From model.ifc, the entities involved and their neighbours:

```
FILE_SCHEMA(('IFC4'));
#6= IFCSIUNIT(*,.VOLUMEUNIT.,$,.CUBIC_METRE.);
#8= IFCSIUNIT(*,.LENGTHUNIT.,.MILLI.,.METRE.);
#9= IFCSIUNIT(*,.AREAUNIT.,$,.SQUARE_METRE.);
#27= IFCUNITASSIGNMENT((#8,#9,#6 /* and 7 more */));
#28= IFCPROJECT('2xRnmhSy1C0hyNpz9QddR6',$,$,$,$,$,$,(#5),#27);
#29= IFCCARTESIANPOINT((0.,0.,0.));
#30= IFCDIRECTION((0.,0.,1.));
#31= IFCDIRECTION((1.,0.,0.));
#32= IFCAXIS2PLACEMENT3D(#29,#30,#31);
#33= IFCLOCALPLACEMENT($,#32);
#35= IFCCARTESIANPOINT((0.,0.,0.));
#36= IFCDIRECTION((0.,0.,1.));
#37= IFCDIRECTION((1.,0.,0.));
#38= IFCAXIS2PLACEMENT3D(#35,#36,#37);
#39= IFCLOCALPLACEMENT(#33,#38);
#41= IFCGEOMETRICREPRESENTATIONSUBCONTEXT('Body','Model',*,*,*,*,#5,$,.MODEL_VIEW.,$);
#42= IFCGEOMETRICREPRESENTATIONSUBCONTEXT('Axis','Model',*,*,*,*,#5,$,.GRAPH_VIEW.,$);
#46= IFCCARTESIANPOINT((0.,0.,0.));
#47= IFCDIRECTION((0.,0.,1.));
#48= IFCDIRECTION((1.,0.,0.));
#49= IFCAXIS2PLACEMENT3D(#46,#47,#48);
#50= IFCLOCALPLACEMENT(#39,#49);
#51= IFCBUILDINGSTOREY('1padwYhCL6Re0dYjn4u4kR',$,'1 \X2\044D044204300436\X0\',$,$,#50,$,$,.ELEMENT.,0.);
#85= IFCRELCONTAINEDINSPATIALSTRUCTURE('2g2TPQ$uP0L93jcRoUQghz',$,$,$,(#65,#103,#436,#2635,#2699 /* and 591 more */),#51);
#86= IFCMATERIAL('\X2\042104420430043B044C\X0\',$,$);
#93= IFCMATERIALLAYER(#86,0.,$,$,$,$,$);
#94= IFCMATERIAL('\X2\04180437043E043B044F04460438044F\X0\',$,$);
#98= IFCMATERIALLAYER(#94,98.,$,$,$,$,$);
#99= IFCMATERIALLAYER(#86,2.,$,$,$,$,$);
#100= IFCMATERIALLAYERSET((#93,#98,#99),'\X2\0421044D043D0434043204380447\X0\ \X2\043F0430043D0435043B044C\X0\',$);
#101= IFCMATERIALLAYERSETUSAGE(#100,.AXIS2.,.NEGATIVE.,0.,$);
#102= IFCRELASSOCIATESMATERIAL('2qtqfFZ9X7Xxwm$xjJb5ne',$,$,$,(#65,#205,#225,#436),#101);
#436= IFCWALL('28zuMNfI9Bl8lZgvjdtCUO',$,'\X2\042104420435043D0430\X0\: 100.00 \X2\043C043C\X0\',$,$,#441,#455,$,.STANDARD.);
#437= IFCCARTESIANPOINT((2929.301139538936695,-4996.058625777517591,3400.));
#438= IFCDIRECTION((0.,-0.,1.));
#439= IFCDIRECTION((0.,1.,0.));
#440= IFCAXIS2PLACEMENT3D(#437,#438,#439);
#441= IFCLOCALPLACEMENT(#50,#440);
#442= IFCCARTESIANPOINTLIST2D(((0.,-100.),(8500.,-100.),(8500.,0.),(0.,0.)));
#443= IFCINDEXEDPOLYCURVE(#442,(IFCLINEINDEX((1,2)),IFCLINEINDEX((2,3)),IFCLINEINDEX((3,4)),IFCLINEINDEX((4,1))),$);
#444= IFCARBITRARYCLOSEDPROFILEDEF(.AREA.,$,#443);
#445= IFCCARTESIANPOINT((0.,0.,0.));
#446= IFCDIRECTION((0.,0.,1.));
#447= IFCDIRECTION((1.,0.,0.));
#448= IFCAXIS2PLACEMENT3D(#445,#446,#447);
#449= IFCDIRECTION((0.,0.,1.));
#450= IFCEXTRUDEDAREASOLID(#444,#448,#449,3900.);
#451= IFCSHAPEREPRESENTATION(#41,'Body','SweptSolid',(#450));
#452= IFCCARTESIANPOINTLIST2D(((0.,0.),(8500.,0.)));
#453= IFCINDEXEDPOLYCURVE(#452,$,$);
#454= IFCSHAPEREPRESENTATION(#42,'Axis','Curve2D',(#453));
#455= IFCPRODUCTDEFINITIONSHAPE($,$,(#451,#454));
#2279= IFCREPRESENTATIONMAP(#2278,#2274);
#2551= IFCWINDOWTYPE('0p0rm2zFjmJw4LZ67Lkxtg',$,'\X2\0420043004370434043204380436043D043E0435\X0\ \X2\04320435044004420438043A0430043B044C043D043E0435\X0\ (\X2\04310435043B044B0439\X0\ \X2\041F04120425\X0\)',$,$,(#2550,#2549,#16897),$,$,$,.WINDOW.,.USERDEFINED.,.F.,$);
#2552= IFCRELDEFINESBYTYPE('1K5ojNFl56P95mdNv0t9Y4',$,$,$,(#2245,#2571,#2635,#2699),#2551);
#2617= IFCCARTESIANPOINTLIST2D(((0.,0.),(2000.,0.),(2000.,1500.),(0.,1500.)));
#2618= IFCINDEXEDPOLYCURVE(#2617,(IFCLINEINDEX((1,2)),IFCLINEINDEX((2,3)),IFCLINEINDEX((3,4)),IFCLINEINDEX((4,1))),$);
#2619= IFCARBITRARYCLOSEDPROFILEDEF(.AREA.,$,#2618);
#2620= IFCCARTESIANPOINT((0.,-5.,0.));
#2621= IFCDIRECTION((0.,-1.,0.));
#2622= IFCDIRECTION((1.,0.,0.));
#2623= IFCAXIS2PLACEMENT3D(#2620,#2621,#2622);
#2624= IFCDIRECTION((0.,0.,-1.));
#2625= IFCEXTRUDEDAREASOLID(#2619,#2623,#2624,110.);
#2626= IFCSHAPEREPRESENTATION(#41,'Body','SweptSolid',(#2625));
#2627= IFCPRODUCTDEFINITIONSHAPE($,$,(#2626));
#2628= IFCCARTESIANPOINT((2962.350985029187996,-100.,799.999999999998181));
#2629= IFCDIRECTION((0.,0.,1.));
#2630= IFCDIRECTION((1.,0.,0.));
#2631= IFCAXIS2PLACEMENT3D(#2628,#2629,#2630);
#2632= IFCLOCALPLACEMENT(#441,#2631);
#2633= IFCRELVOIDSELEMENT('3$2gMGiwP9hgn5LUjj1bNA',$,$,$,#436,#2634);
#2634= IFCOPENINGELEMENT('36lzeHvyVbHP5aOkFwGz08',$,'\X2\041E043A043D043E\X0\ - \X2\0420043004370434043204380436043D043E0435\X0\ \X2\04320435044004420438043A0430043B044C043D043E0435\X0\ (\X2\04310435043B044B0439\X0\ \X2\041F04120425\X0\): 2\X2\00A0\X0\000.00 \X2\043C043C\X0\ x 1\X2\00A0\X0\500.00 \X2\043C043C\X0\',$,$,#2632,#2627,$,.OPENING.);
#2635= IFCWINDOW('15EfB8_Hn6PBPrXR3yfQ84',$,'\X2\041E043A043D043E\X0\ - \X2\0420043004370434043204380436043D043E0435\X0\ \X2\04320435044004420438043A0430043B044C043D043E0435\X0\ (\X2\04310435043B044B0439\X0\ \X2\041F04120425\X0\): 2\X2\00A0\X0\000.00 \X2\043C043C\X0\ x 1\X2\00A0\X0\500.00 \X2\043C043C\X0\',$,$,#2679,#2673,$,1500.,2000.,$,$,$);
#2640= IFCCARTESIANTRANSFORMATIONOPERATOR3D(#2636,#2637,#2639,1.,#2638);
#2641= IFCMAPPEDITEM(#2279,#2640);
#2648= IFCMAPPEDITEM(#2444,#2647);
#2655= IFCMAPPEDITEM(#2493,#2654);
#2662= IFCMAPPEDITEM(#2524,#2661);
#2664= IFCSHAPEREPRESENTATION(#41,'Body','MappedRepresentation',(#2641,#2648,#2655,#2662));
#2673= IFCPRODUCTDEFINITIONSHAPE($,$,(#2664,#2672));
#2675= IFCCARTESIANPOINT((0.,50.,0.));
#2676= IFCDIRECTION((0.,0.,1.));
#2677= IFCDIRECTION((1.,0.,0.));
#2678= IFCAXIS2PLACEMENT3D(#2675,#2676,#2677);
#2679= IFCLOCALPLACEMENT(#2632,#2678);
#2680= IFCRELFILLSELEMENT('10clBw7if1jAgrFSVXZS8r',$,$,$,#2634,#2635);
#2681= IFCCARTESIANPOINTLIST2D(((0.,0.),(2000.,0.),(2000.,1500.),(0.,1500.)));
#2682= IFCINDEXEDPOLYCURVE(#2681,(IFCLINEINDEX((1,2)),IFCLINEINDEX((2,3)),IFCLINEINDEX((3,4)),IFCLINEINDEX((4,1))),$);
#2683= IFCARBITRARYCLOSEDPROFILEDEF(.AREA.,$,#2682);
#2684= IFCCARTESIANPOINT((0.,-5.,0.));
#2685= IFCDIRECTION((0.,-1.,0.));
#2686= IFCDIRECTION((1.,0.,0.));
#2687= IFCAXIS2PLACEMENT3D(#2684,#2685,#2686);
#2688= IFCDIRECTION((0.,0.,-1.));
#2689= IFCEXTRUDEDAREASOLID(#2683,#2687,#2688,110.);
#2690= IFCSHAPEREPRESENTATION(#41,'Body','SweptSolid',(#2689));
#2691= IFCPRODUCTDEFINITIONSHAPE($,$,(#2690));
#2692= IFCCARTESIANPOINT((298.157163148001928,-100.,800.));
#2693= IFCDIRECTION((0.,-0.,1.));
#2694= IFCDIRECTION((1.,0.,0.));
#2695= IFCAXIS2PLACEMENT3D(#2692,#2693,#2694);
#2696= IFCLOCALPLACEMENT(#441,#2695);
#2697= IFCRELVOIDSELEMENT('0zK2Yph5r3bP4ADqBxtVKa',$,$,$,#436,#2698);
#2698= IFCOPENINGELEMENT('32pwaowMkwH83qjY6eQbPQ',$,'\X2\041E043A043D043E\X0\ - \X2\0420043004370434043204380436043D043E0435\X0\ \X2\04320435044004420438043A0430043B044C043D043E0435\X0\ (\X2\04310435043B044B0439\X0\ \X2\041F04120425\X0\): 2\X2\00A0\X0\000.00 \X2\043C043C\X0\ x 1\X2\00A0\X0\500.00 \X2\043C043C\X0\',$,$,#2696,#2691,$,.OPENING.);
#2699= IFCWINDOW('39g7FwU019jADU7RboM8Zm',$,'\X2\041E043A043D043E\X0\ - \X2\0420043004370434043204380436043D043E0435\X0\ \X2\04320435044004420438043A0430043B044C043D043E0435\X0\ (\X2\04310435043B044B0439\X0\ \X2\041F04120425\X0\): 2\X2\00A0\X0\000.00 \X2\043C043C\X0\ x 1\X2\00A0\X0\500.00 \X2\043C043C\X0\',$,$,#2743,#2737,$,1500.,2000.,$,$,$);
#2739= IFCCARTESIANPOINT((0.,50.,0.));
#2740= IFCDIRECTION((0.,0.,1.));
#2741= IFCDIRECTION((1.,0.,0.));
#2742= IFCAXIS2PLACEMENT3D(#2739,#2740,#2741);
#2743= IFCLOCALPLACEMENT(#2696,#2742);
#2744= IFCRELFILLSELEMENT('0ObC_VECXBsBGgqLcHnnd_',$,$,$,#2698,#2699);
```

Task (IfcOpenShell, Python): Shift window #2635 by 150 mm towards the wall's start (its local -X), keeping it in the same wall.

```python
import ifcopenshell
import ifcopenshell.api.geometry
import ifcopenshell.util.placement
import ifcopenshell.util.unit

model = ifcopenshell.open("model.ifc")
unit_scale = ifcopenshell.util.unit.calculate_unit_scale(model)

window = model.by_id(2635)
opening = window.FillsVoids[0].RelatingOpeningElement
wall = opening.VoidsElements[0].RelatingBuildingElement

wall_matrix = ifcopenshell.util.placement.get_local_placement(wall.ObjectPlacement)
shift = wall_matrix[:3, 0] * -0.15 / unit_scale
before = ifcopenshell.util.placement.get_local_placement(window.ObjectPlacement)[:3, 3].copy()

# The window is placed relative to its opening, so it follows when the opening moves.
matrix = ifcopenshell.util.placement.get_local_placement(opening.ObjectPlacement)
matrix[:3, 3] += shift
ifcopenshell.api.geometry.edit_object_placement(
    model, product=opening, matrix=matrix, is_si=False, should_transform_children=True
)

after = ifcopenshell.util.placement.get_local_placement(window.ObjectPlacement)[:3, 3]
print("window moved by", (after - before).round(3) + 0.0)

model.write("model_v2.ifc")
```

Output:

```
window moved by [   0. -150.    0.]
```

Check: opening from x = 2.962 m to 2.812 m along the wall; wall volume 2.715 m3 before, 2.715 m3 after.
